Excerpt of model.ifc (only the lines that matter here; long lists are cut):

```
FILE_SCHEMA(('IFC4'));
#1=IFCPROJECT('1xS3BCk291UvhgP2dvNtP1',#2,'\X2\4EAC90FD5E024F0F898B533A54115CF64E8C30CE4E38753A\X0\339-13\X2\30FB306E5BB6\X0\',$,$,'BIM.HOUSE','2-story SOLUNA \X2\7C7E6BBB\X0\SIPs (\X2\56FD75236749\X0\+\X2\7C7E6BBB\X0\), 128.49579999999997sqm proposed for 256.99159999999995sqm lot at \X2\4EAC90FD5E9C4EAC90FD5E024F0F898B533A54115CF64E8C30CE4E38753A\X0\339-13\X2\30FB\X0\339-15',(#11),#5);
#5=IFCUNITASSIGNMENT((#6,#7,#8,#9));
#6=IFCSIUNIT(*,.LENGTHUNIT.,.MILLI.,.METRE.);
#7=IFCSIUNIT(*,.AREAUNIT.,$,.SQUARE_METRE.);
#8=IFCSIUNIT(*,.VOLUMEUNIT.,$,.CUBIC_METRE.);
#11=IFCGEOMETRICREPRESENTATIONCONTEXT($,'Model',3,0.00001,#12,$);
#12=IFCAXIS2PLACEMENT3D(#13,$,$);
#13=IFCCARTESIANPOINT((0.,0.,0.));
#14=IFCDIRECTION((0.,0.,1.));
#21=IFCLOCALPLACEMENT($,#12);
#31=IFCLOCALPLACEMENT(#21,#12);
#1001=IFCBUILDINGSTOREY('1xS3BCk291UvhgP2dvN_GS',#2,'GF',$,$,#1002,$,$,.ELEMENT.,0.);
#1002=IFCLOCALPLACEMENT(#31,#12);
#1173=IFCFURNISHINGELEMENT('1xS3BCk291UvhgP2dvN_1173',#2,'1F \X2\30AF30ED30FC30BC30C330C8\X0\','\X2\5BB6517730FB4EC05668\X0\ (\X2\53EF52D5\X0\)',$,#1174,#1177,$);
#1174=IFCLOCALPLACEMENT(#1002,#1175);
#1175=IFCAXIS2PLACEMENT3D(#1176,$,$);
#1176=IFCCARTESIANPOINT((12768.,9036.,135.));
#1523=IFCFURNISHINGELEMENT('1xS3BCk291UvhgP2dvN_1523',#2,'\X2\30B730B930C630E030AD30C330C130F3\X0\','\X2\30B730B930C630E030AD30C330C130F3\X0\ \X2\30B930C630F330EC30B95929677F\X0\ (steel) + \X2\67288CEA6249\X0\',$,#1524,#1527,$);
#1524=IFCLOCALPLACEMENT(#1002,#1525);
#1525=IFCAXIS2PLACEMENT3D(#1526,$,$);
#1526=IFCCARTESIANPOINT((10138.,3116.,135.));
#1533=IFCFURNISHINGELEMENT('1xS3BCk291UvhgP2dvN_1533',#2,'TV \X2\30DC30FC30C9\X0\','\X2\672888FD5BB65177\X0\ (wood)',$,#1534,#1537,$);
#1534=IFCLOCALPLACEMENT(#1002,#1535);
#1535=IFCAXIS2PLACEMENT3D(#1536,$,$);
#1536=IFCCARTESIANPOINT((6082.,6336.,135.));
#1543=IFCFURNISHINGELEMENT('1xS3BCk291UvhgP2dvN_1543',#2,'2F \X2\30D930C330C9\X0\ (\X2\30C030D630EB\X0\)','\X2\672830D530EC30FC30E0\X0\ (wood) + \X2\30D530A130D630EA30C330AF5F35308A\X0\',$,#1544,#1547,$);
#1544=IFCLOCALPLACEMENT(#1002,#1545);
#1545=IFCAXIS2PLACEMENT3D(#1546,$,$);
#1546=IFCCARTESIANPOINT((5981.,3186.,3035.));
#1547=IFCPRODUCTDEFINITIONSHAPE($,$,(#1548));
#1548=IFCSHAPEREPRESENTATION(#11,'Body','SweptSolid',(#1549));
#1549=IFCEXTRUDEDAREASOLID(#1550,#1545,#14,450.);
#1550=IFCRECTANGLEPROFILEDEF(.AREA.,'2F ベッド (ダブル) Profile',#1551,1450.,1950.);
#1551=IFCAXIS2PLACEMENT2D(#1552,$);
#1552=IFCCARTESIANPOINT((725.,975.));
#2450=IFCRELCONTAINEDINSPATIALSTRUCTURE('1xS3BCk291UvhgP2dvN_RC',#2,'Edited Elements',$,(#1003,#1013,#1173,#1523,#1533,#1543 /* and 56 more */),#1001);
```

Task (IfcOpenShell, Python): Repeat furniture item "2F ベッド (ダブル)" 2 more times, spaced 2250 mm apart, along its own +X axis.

```python
import ifcopenshell
import ifcopenshell.api.geometry
import ifcopenshell.api.root
import ifcopenshell.util.element
import ifcopenshell.util.placement
import ifcopenshell.util.unit

model = ifcopenshell.open("model.ifc")
unit_scale = ifcopenshell.util.unit.calculate_unit_scale(model)


def reuse_history(source, copy):
    """copy_class also copies each property set's owner history, people and application; keep the originals."""
    for rel in copy.IsDefinedBy:
        if rel.is_a("IfcRelDefinesByProperties") and (history := rel.RelatingPropertyDefinition.OwnerHistory):
            rel.RelatingPropertyDefinition.OwnerHistory = source.OwnerHistory
            ifcopenshell.util.element.remove_deep2(model, history)


source = model.by_id(1543)
base = ifcopenshell.util.placement.get_local_placement(source.ObjectPlacement)
step = base[:3, 0] * 2.25 / unit_scale

for i in range(1, 3):
    copy = ifcopenshell.api.root.copy_class(model, product=source)
    copy.Representation = ifcopenshell.util.element.copy_deep(
        model, source.Representation, exclude=["IfcGeometricRepresentationContext", "IfcRepresentationMap"]
    )
    reuse_history(source, copy)
    matrix = base.copy()
    matrix[:3, 3] += i * step
    print("added at", matrix[:3, 3].round(3) + 0.0)
    ifcopenshell.api.geometry.edit_object_placement(model, product=copy, matrix=matrix, is_si=False)

model.write("model_updated.ifc")
```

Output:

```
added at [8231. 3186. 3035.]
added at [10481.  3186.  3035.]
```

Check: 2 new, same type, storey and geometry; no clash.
